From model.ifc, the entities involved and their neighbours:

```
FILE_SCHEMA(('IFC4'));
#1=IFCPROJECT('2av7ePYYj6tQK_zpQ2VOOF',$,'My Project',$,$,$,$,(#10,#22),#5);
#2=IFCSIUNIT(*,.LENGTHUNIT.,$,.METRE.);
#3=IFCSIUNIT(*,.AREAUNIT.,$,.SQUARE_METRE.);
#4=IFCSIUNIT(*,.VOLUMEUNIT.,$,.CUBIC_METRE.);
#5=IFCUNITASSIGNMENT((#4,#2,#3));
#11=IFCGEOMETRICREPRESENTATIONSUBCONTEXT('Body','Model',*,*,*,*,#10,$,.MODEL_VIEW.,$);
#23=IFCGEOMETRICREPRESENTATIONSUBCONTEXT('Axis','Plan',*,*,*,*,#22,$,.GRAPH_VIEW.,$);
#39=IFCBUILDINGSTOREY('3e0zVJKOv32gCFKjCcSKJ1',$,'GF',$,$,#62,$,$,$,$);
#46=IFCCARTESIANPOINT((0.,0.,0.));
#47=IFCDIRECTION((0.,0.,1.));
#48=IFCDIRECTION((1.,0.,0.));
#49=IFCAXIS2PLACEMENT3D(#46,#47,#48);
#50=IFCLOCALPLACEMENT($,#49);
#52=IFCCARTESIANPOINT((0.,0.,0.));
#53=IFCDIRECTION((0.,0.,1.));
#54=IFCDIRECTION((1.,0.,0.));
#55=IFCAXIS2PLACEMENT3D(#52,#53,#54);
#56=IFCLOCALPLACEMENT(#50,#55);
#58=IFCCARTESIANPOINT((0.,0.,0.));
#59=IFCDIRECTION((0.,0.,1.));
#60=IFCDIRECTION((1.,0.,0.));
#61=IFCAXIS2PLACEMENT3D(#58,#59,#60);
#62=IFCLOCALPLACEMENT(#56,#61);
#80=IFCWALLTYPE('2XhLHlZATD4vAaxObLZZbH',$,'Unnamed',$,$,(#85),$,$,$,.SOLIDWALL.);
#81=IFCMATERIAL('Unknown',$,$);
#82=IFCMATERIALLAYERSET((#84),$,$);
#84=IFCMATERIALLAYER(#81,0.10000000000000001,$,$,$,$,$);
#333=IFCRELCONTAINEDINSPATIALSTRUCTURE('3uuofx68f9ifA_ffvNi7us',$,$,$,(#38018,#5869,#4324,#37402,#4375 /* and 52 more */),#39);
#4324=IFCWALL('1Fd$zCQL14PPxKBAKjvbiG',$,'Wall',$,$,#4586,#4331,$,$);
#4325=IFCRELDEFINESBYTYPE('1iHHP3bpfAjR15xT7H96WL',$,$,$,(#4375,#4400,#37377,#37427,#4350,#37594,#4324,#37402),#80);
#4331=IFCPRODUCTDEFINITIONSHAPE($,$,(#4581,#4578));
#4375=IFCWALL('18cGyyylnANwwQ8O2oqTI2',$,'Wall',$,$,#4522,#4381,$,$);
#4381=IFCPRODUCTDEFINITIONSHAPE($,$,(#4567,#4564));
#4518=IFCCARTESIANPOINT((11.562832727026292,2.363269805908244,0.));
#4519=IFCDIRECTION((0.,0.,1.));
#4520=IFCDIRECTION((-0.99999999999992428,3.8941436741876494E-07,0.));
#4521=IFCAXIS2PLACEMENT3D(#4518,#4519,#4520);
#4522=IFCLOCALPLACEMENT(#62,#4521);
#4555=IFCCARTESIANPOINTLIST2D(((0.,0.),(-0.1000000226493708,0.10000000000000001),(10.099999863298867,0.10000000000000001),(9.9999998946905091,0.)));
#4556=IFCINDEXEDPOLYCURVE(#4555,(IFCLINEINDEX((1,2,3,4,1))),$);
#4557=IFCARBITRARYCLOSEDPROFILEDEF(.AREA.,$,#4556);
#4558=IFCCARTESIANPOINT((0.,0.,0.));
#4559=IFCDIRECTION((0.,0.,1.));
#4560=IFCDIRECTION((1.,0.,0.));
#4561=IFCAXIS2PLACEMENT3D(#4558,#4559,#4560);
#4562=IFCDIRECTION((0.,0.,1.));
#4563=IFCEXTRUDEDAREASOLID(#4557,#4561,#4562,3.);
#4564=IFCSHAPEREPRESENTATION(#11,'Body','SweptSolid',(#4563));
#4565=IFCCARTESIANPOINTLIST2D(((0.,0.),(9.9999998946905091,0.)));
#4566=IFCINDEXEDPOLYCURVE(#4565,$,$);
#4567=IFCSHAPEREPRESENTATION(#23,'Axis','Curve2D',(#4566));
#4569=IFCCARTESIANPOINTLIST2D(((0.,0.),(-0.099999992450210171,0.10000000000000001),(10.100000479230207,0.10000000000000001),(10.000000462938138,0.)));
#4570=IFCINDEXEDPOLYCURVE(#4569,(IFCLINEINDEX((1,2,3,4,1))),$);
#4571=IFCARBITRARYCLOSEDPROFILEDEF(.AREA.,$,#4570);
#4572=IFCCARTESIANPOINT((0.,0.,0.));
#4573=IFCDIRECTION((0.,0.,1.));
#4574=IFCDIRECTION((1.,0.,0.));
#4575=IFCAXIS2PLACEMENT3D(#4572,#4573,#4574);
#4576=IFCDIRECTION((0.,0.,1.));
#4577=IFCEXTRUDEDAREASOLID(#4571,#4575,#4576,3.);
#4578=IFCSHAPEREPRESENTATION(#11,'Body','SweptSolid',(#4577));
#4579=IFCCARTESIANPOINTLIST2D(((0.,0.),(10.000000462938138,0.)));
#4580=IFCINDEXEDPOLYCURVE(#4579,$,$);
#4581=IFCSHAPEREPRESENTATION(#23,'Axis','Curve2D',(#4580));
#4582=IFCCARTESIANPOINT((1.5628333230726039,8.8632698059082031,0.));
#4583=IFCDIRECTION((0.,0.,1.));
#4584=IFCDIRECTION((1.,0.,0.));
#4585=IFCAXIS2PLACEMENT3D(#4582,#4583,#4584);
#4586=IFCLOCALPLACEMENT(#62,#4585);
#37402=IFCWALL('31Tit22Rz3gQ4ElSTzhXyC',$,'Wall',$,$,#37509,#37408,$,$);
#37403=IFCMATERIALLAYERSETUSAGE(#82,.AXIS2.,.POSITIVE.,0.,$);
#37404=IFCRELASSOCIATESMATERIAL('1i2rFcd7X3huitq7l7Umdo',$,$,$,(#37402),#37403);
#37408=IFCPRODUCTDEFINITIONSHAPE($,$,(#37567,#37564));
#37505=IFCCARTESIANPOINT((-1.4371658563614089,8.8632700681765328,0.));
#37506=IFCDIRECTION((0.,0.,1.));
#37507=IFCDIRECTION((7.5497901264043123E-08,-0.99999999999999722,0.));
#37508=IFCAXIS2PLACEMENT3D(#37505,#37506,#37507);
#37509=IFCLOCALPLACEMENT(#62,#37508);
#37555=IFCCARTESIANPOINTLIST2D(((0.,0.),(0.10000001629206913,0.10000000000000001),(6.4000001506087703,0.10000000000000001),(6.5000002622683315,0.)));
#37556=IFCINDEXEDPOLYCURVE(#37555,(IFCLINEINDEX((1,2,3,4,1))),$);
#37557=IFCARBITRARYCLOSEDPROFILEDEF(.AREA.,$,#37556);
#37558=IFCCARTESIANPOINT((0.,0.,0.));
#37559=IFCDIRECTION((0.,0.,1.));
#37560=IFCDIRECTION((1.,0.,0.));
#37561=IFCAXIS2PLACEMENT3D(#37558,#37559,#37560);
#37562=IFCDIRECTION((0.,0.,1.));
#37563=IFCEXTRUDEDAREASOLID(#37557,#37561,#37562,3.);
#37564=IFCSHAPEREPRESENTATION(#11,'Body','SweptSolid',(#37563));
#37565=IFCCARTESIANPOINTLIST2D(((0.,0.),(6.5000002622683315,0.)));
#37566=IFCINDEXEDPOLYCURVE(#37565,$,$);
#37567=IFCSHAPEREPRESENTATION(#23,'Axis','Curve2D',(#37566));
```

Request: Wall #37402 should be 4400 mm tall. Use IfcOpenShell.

```python
import ifcopenshell
import ifcopenshell.geom
import ifcopenshell.util.representation
import ifcopenshell.util.shape
import ifcopenshell.util.unit

model = ifcopenshell.open("model.ifc")
unit_scale = ifcopenshell.util.unit.calculate_unit_scale(model)
settings = ifcopenshell.geom.settings()


def volume(element):
    """Net volume in cubic metres, openings subtracted."""
    shape = ifcopenshell.geom.create_shape(settings, element)
    return ifcopenshell.util.shape.get_volume(shape.geometry)


wall = model.by_guid("31Tit22Rz3gQ4ElSTzhXyC")
before = volume(wall)

body = ifcopenshell.util.representation.get_representation(wall, "Model", "Body")
solid = body.Items[0]
old_height = solid.Depth
solid.Depth = 4.4 / unit_scale
after = volume(wall)

print(f"height {old_height:g} -> {solid.Depth:g}, volume {before:.3f} -> {after:.3f} m3")

model.write("model_updated.ifc")
```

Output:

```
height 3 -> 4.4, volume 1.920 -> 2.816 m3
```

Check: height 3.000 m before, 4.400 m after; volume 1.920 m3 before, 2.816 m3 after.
